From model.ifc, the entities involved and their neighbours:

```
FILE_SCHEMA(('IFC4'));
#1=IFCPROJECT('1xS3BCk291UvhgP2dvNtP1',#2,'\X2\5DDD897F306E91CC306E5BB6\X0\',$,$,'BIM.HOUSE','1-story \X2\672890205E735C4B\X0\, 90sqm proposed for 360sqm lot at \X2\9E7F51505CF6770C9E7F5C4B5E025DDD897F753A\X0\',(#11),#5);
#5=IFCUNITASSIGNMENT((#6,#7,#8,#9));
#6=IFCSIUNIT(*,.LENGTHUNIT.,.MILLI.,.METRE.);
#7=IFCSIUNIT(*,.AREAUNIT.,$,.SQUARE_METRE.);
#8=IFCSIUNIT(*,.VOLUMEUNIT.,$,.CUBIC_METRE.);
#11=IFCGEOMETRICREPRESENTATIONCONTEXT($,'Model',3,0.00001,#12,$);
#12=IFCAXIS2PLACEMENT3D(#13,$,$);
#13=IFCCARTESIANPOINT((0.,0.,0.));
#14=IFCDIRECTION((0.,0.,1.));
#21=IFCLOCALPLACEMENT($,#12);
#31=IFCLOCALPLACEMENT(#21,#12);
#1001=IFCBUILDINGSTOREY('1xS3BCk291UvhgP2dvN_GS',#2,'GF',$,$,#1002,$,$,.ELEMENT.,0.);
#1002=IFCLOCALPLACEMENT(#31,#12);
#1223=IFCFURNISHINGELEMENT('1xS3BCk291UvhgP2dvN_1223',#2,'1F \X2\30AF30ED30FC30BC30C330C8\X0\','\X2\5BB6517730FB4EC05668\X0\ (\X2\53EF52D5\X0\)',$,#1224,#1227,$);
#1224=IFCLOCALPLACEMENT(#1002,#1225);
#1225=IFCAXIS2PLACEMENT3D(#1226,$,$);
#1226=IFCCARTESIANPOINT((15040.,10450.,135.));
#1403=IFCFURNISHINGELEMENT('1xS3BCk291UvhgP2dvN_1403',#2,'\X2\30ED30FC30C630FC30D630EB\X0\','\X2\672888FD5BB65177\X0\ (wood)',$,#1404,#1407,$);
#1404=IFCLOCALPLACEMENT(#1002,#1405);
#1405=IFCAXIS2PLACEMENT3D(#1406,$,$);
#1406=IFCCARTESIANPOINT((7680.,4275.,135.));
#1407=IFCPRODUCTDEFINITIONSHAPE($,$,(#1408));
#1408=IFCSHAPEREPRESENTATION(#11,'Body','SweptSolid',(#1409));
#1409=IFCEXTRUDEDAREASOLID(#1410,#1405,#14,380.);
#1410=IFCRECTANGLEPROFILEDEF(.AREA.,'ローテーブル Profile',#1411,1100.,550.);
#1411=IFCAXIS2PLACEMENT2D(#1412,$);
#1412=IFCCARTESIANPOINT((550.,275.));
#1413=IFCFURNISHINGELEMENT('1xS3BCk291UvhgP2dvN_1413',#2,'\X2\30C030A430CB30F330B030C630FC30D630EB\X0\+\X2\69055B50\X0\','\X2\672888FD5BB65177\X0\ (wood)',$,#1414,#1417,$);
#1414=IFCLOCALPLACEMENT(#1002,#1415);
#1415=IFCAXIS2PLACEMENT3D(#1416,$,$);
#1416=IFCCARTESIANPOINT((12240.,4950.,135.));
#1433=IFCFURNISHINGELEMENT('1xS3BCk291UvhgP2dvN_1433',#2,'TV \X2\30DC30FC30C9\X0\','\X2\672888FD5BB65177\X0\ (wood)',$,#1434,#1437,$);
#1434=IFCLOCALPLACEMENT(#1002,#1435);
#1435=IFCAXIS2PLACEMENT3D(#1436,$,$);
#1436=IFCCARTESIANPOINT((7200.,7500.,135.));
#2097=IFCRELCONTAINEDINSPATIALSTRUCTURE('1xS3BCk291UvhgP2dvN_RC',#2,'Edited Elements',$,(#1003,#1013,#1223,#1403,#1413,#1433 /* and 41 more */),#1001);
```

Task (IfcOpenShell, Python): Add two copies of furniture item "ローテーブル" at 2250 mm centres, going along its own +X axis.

```python
import ifcopenshell
import ifcopenshell.api.geometry
import ifcopenshell.api.root
import ifcopenshell.util.element
import ifcopenshell.util.placement

model = ifcopenshell.open("model.ifc")


def reuse_history(source, copy):
    """copy_class also copies each property set's owner history, people and application; keep the originals."""
    for rel in copy.IsDefinedBy:
        if rel.is_a("IfcRelDefinesByProperties") and (history := rel.RelatingPropertyDefinition.OwnerHistory):
            rel.RelatingPropertyDefinition.OwnerHistory = source.OwnerHistory
            ifcopenshell.util.element.remove_deep2(model, history)


source = model.by_guid("1xS3BCk291UvhgP2dvN_1403")
base = ifcopenshell.util.placement.get_local_placement(source.ObjectPlacement)
step = base[:3, 0] * 2250.0

for i in range(1, 3):
    copy = ifcopenshell.api.root.copy_class(model, product=source)
    copy.Representation = ifcopenshell.util.element.copy_deep(
        model, source.Representation, exclude=["IfcGeometricRepresentationContext", "IfcRepresentationMap"]
    )
    reuse_history(source, copy)
    matrix = base.copy()
    matrix[:3, 3] += i * step
    print("added at", matrix[:3, 3].round(3) + 0.0)
    ifcopenshell.api.geometry.edit_object_placement(model, product=copy, matrix=matrix, is_si=False)

model.write("model-out.ifc")
```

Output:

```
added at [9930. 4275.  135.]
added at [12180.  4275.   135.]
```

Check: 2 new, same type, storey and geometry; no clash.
